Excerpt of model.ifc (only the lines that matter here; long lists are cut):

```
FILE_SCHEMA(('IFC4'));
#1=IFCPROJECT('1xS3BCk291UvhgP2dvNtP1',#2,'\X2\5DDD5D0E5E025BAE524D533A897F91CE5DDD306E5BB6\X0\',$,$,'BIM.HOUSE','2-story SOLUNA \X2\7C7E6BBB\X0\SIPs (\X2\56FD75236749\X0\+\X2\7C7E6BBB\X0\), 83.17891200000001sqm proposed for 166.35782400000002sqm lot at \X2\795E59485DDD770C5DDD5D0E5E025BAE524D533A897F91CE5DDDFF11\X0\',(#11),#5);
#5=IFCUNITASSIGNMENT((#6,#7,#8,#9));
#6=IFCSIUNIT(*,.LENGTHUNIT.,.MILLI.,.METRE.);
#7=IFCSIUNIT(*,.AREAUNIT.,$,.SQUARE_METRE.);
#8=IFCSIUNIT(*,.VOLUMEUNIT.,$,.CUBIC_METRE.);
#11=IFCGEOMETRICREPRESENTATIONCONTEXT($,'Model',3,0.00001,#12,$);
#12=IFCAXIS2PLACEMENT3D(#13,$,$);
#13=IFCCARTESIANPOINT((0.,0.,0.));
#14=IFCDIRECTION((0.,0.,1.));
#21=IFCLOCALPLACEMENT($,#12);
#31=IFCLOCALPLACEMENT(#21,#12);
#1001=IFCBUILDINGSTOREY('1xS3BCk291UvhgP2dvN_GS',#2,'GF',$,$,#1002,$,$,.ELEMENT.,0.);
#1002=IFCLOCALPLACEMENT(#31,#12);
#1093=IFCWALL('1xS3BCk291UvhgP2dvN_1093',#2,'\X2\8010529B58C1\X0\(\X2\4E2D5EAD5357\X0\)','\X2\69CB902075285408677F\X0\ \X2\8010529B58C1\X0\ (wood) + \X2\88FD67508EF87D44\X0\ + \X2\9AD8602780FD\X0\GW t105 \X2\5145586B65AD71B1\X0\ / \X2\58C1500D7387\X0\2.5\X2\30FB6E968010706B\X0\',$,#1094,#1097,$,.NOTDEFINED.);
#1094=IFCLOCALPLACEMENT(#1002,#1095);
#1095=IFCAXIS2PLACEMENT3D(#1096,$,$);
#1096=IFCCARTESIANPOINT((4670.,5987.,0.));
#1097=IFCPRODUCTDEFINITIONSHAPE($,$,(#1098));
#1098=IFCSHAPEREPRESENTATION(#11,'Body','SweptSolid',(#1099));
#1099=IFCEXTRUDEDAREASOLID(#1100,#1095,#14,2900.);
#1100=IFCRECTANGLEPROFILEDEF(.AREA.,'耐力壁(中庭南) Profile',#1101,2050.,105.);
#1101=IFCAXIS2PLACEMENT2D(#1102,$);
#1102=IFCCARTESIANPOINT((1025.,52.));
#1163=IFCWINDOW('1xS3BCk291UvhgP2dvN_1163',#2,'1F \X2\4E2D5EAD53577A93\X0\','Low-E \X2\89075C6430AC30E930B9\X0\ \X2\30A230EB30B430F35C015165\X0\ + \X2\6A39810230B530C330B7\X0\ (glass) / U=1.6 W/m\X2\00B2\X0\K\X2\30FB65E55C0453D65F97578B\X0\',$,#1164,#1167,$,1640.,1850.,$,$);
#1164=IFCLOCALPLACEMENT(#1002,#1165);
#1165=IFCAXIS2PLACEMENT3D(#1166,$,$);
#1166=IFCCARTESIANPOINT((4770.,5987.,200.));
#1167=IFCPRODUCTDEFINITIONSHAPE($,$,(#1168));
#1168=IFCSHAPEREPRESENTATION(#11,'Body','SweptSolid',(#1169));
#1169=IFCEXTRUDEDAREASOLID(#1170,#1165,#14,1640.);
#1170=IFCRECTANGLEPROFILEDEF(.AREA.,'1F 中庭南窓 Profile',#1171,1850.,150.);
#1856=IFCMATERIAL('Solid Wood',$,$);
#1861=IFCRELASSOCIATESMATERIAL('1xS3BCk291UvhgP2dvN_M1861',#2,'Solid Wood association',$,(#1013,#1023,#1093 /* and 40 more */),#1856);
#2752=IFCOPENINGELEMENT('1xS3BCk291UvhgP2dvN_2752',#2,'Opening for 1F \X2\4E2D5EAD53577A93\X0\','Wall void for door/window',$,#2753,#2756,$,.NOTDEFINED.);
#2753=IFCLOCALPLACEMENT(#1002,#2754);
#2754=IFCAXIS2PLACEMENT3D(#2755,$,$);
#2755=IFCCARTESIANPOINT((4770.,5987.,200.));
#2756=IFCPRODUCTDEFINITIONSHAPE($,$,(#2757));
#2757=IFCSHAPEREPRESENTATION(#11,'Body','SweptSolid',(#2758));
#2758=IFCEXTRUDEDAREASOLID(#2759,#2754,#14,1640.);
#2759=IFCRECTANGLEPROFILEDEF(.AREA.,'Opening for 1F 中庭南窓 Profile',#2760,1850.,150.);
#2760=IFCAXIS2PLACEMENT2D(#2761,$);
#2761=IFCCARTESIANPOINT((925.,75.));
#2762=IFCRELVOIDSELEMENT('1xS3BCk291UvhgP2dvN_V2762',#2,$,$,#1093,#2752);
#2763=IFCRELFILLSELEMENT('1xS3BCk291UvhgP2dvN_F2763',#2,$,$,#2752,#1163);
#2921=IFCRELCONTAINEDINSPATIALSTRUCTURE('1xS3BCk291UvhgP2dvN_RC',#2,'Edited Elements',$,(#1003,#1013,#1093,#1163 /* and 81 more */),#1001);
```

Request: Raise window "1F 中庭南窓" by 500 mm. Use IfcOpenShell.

```python
import numpy as np
import ifcopenshell
import ifcopenshell.api.geometry
import ifcopenshell.util.placement
import ifcopenshell.util.unit

model = ifcopenshell.open("model.ifc")
unit_scale = ifcopenshell.util.unit.calculate_unit_scale(model)

window = model.by_id(1163)
opening = window.FillsVoids[0].RelatingOpeningElement
dz = 0.5 / unit_scale

shift = np.array([0.0, 0.0, dz])
# The window is not placed relative to its opening, so move both.
for product in (opening, window):
    matrix = ifcopenshell.util.placement.get_local_placement(product.ObjectPlacement)
    matrix[:3, 3] += shift
    ifcopenshell.api.geometry.edit_object_placement(model, product=product, matrix=matrix, is_si=False)

print(f"moved by {dz * unit_scale:+.3f} m")

model.write("model_updated.ifc")
```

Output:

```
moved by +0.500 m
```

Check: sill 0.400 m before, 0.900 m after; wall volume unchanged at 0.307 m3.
